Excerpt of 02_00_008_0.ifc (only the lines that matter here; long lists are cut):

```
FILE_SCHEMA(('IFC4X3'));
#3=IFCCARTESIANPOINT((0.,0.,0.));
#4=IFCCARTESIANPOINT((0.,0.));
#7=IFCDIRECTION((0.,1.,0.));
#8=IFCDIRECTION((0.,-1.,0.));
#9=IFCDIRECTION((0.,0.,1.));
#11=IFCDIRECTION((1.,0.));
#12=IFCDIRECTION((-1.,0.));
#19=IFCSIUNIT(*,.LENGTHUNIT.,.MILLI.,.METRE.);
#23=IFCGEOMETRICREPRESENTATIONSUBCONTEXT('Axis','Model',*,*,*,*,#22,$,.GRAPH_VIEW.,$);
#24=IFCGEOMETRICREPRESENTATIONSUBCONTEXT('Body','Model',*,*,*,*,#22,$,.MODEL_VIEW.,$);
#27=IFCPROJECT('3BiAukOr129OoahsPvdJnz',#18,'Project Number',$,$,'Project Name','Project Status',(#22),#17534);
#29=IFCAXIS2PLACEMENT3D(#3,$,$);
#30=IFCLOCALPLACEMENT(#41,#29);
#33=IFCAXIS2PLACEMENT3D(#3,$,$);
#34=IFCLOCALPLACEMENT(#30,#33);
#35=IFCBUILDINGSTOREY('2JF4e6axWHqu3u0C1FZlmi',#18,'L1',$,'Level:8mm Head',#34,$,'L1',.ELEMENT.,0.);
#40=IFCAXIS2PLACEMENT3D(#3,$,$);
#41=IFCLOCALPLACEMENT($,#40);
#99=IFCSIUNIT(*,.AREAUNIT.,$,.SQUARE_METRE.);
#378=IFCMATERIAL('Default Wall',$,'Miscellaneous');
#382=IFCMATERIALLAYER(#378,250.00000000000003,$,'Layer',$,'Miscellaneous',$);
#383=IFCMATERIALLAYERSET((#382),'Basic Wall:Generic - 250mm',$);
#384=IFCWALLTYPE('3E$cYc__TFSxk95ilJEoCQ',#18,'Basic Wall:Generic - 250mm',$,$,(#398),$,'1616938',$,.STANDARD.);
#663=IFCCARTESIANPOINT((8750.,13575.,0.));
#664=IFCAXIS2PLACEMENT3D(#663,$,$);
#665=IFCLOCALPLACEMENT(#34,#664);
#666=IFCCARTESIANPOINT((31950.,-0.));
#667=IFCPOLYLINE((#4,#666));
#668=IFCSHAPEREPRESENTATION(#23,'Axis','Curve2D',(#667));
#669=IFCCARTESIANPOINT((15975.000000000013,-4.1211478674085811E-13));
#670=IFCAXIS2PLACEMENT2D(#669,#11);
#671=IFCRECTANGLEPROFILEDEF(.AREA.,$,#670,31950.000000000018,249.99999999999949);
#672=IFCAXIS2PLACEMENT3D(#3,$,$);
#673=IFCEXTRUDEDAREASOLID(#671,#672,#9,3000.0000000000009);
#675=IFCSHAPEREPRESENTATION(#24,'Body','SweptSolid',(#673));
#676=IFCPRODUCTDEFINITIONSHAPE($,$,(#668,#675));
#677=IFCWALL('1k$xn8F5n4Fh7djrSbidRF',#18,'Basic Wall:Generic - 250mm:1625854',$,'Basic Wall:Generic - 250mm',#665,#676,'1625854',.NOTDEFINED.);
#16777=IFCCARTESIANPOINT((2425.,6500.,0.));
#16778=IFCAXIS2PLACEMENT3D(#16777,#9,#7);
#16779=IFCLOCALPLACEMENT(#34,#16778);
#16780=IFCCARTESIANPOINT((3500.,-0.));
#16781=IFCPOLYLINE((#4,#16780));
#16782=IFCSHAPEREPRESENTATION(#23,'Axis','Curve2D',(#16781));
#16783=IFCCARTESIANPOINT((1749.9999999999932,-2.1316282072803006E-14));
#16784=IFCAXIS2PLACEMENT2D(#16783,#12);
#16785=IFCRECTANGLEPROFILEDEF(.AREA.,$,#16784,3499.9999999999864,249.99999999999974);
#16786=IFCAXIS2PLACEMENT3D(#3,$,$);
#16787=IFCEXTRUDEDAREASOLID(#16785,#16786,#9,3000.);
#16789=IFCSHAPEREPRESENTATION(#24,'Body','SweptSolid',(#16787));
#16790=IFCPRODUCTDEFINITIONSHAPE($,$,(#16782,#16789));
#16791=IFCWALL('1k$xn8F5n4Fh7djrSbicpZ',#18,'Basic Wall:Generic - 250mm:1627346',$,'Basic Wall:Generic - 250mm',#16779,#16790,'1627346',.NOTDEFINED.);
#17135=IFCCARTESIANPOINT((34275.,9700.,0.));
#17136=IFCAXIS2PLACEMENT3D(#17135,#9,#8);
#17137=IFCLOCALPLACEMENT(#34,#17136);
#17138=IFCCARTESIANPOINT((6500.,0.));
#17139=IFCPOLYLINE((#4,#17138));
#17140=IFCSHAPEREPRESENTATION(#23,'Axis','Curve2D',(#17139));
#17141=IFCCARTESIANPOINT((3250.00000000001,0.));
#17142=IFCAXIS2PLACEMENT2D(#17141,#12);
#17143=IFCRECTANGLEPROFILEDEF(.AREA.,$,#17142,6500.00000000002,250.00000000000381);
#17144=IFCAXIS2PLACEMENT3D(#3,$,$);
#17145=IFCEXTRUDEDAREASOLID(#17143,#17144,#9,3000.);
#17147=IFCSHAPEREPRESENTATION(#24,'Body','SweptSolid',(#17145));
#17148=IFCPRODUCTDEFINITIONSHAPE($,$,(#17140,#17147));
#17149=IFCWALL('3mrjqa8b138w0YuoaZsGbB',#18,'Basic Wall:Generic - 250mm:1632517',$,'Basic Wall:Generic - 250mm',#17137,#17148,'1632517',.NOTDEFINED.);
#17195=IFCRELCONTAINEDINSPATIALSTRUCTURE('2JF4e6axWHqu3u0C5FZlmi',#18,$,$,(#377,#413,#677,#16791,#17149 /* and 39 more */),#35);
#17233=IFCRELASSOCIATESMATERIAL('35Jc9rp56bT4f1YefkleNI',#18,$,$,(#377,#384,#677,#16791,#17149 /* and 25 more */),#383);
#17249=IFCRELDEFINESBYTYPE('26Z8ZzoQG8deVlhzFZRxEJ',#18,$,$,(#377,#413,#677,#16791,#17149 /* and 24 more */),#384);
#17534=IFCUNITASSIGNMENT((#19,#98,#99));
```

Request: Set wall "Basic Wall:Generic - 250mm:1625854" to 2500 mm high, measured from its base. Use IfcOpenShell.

```python
import ifcopenshell
import ifcopenshell.geom
import ifcopenshell.util.representation
import ifcopenshell.util.shape
import ifcopenshell.util.unit

model = ifcopenshell.open("02_00_008_0.ifc")
unit_scale = ifcopenshell.util.unit.calculate_unit_scale(model)
settings = ifcopenshell.geom.settings()


def volume(element):
    """Net volume in cubic metres, openings subtracted."""
    shape = ifcopenshell.geom.create_shape(settings, element)
    return ifcopenshell.util.shape.get_volume(shape.geometry)


wall = model.by_guid("1k$xn8F5n4Fh7djrSbidRF")
before = volume(wall)

body = ifcopenshell.util.representation.get_representation(wall, "Model", "Body")
solid = body.Items[0]
old_height = solid.Depth
solid.Depth = 2.5 / unit_scale
after = volume(wall)

print(f"height {old_height:g} -> {solid.Depth:g}, volume {before:.3f} -> {after:.3f} m3")

model.write("02_00_008_0_v2.ifc")
```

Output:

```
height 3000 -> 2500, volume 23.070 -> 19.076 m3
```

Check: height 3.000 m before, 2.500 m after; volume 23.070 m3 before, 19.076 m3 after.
